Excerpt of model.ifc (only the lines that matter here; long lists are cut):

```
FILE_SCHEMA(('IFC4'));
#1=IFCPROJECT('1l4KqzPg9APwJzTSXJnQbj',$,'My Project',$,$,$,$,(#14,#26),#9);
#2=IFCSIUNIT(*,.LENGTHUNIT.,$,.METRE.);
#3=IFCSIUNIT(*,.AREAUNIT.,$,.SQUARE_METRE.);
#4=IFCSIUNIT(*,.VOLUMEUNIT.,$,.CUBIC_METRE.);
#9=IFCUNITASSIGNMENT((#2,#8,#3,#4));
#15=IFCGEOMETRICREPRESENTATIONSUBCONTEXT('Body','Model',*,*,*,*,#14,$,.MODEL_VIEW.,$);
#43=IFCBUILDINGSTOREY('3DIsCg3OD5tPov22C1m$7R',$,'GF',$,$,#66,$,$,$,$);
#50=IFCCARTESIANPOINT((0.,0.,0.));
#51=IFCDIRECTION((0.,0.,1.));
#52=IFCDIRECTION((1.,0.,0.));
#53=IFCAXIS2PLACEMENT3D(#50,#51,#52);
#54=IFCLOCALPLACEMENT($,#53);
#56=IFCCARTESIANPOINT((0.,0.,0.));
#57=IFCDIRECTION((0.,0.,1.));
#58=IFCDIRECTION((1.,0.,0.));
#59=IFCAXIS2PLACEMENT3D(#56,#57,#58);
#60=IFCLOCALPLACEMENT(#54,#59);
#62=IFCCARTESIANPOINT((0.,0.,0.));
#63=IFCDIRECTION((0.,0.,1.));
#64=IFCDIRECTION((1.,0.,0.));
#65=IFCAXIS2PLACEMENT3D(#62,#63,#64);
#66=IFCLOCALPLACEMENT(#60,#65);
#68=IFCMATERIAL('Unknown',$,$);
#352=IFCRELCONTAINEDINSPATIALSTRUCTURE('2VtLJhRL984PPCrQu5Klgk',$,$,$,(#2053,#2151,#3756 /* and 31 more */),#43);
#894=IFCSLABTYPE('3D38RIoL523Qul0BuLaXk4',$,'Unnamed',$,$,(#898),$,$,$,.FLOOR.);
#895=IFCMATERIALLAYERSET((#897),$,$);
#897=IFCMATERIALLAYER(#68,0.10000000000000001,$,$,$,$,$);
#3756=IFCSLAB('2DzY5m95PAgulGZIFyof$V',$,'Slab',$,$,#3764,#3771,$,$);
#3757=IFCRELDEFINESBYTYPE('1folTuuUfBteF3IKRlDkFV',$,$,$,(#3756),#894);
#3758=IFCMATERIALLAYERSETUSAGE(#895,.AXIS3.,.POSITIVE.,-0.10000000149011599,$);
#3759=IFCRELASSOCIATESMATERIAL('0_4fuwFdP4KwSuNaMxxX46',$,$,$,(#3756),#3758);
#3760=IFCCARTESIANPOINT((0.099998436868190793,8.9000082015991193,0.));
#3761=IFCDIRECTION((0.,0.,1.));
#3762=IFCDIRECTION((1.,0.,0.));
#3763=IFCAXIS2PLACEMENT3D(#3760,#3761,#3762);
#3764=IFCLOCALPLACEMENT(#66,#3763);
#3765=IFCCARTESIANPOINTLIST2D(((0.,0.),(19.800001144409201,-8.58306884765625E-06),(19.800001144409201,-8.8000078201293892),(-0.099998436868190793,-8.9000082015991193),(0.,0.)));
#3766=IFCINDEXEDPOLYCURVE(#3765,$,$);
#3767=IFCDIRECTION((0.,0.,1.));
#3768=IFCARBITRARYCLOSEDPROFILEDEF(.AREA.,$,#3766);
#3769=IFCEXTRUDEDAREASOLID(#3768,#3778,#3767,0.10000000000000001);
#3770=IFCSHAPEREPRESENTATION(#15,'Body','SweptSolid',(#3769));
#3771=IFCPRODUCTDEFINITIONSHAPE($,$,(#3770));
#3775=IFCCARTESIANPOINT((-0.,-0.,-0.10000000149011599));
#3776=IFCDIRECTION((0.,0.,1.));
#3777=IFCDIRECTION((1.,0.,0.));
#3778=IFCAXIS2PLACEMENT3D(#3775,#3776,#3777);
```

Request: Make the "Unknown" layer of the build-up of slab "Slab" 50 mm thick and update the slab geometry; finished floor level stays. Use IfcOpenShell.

```python
import ifcopenshell
import ifcopenshell.util.element
import ifcopenshell.util.representation
import ifcopenshell.util.unit

model = ifcopenshell.open("model.ifc")
unit_scale = ifcopenshell.util.unit.calculate_unit_scale(model)

layer_set = model.by_id(895)
layer = next(l for l in layer_set.MaterialLayers if l.Material and l.Material.Name == "Unknown")
change = 0.05 / unit_scale - layer.LayerThickness
layer.LayerThickness += change

# Geometry does not follow the layer set by itself.
slabs = [e for e in ifcopenshell.util.element.get_elements_by_material(model, layer_set) if e.is_a("IfcSlab")]
for slab in sorted(slabs, key=lambda e: e.id()):
    body = ifcopenshell.util.representation.get_representation(slab, "Model", "Body")
    solid = body.Items[0]
    old_depth = solid.Depth
    solid.Depth += change
    # Extruded upwards: lower the start of the extrusion so the top stays.
    x, y, z = solid.Position.Location.Coordinates
    solid.Position.Location = model.createIfcCartesianPoint((x, y, z - change))
    print(slab.id(), f"{old_depth:g} -> {solid.Depth:g}")

# The layers are counted up from the underside, which has moved.
for usage in {ifcopenshell.util.element.get_material(slab) for slab in slabs}:
    usage.OffsetFromReferenceLine -= change

model.write("model_edited.ifc")
```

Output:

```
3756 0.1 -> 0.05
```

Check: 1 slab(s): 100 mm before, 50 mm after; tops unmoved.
